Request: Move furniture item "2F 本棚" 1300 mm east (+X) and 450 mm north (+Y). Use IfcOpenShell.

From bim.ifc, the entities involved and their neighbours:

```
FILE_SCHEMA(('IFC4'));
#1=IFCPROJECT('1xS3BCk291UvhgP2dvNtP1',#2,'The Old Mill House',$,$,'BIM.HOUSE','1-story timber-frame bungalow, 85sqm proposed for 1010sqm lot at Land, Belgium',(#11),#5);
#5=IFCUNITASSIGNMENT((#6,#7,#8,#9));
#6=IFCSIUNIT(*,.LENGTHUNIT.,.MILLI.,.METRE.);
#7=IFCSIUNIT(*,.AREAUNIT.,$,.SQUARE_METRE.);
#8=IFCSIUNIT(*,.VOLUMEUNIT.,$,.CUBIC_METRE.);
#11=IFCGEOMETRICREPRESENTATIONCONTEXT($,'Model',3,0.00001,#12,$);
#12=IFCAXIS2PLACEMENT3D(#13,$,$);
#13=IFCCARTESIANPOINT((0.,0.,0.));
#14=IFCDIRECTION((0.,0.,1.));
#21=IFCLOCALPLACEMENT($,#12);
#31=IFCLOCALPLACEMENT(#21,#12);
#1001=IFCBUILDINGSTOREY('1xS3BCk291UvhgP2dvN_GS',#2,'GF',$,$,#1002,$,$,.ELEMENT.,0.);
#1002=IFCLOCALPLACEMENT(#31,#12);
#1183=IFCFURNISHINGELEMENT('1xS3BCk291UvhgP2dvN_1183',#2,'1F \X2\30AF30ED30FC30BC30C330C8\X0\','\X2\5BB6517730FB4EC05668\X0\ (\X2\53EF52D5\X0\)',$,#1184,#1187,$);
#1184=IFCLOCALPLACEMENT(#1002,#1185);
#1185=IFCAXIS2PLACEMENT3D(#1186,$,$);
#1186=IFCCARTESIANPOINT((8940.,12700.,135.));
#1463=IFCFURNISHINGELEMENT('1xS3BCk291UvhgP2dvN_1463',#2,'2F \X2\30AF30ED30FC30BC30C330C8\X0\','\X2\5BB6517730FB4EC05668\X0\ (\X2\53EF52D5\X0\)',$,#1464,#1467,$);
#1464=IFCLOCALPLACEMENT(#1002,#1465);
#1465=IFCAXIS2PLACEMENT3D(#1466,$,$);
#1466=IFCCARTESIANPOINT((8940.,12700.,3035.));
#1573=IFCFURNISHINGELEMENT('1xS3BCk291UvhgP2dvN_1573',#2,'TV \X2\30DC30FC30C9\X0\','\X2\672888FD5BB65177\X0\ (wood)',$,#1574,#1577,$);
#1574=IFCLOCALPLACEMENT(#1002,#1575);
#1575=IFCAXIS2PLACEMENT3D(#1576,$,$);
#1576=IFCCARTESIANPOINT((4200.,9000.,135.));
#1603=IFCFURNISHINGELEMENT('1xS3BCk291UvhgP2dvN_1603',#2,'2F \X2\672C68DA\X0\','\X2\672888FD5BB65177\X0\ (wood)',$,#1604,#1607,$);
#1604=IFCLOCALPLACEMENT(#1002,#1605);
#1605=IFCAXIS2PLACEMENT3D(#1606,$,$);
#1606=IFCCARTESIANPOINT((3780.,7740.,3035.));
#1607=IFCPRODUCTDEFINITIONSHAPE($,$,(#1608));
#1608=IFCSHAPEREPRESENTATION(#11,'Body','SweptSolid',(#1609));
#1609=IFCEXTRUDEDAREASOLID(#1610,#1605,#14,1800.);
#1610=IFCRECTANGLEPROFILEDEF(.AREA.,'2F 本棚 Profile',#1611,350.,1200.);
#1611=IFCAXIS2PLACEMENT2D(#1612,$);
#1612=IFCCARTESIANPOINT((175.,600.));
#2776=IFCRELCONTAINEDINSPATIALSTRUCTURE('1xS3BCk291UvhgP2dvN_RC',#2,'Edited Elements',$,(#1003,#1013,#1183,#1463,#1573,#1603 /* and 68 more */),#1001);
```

```python
import ifcopenshell
import ifcopenshell.api.geometry
import ifcopenshell.util.placement

model = ifcopenshell.open("bim.ifc")

item = model.by_guid("1xS3BCk291UvhgP2dvN_1603")
matrix = ifcopenshell.util.placement.get_local_placement(item.ObjectPlacement)
matrix[0, 3] += 1300.0
matrix[1, 3] += 450.0
ifcopenshell.api.geometry.edit_object_placement(model, product=item, matrix=matrix, is_si=False)

print(ifcopenshell.util.placement.get_local_placement(item.ObjectPlacement).round(3) + 0.0)

model.write("bim-out.ifc")
```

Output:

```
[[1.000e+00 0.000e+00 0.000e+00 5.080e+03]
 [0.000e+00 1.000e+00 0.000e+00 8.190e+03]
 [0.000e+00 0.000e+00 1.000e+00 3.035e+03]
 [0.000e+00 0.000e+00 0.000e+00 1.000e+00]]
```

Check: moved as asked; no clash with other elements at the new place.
